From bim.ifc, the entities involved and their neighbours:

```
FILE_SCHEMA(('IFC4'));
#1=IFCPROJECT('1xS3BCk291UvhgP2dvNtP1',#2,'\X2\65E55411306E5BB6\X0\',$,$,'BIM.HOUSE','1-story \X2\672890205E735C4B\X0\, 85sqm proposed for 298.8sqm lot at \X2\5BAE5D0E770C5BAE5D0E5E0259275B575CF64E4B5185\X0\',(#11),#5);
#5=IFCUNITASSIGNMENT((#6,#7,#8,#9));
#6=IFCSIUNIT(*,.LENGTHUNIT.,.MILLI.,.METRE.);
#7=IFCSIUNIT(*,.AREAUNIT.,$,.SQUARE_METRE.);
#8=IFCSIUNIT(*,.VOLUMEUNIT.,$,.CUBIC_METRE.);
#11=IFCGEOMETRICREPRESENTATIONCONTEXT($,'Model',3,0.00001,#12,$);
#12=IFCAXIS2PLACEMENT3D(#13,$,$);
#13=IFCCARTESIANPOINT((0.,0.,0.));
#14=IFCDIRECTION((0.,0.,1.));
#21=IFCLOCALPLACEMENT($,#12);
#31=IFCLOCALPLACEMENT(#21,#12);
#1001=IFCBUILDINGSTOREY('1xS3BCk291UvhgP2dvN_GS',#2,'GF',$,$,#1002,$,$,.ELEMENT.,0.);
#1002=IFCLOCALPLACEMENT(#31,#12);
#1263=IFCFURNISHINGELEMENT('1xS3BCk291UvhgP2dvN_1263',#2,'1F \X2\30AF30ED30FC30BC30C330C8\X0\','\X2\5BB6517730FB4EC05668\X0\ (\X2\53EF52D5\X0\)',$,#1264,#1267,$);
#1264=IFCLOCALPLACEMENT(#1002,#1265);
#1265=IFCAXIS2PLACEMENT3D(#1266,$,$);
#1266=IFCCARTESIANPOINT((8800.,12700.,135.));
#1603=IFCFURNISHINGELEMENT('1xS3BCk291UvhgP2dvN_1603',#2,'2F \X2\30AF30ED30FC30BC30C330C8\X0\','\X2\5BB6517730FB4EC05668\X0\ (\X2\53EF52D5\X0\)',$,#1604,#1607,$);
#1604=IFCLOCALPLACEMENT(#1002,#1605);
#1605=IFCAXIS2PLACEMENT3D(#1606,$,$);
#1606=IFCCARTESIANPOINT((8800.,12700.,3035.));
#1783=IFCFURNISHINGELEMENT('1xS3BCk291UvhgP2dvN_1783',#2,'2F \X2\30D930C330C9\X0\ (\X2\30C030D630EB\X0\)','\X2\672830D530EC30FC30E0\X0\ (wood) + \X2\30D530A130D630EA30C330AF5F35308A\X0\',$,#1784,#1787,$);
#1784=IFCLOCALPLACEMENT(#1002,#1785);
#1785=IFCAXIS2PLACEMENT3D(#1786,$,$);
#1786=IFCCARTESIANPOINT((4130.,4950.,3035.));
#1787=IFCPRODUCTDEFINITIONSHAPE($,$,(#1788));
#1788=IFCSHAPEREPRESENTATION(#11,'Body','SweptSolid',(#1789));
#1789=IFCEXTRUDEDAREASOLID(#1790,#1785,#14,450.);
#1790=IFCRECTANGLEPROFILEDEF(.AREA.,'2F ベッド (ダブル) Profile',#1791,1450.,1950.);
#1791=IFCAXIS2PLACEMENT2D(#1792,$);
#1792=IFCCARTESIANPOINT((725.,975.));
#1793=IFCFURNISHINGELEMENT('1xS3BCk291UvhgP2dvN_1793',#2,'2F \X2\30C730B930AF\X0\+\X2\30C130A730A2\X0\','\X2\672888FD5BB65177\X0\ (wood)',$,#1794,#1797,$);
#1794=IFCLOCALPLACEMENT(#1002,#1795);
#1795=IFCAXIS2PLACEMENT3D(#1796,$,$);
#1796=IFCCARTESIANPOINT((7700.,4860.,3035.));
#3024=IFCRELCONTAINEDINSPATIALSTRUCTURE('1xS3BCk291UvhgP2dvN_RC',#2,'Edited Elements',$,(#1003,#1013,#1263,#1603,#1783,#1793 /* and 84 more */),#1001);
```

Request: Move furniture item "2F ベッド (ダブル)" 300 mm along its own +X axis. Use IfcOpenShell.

```python
import ifcopenshell
import ifcopenshell.api.geometry
import ifcopenshell.util.placement

model = ifcopenshell.open("bim.ifc")

item = model.by_guid("1xS3BCk291UvhgP2dvN_1783")
matrix = ifcopenshell.util.placement.get_local_placement(item.ObjectPlacement)
matrix[:3, 3] += matrix[:3, 0] * 300.0
ifcopenshell.api.geometry.edit_object_placement(model, product=item, matrix=matrix, is_si=False)

print(ifcopenshell.util.placement.get_local_placement(item.ObjectPlacement).round(3) + 0.0)

model.write("bim_v2.ifc")
```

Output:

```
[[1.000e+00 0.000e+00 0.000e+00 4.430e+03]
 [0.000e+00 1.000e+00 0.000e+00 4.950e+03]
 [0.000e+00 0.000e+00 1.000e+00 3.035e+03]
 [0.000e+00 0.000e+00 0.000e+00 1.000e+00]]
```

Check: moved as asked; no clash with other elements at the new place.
